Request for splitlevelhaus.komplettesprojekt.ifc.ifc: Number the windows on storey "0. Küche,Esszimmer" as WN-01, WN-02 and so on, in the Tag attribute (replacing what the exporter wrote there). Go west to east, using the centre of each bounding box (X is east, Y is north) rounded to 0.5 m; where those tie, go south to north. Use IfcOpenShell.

First a look at what the model holds.

```python
import ifcopenshell
import ifcopenshell.util.element
import ifcopenshell.util.placement

model = ifcopenshell.open("splitlevelhaus.komplettesprojekt.ifc.ifc")
print(model.schema)
storey = next(s for s in model.by_type("IfcBuildingStorey") if s.Name == "0. Küche,Esszimmer")
windows = [e for e in ifcopenshell.util.element.get_decomposition(storey) if e.is_a("IfcWindow")]
for e in sorted(windows, key=lambda e: e.id()):
    origin = ifcopenshell.util.placement.get_local_placement(e.ObjectPlacement)[:3, 3]
    print(e.id(), e.Tag, e.Name, origin.round(2) + 0.0, sep=" | ")
```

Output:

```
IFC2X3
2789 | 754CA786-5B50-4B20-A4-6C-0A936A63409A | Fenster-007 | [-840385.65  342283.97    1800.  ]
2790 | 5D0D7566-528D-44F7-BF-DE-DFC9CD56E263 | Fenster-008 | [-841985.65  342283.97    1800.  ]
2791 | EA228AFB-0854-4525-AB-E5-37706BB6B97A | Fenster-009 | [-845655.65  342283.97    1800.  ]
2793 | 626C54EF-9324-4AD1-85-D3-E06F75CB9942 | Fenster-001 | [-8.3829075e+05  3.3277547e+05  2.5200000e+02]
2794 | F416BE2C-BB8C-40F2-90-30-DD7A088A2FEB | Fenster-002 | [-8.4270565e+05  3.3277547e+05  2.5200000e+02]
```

```python
import ifcopenshell
import ifcopenshell.geom
import ifcopenshell.util.element
import ifcopenshell.util.shape

model = ifcopenshell.open("splitlevelhaus.komplettesprojekt.ifc.ifc")
settings = ifcopenshell.geom.settings()
settings.set("use-world-coords", True)


def centre(element):
    shape = ifcopenshell.geom.create_shape(settings, element)
    return ifcopenshell.util.shape.get_bbox_centroid(shape.geometry)


storey = next(s for s in model.by_type("IfcBuildingStorey") if s.Name == "0. Küche,Esszimmer")
windows = [e for e in ifcopenshell.util.element.get_decomposition(storey) if e.is_a("IfcWindow")]

# Insertion points can sit at a corner or the storey origin, so sort by the geometry (in metres).
centres = {e: centre(e) for e in windows}
windows.sort(key=lambda e: (round(centres[e][0] / 0.5), centres[e][1]))

for i, e in enumerate(windows, start=1):
    number = f"WN-{i:02d}"
    e.Tag = number
    print(e.id(), number)

model.write("splitlevelhaus.komplettesprojekt.ifc_rev.ifc")
```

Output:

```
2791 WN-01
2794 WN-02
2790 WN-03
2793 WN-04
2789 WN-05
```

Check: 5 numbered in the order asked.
